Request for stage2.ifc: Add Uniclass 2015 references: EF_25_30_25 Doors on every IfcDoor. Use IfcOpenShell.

First a look at what the model holds.

```python
import ifcopenshell

model = ifcopenshell.open("stage2.ifc")
print(model.schema)
print("classifications:", [c.Name for c in model.by_type("IfcClassification")])
for ifc_class in ("IfcDoor", "IfcRoof", "IfcStair", "IfcWall", "IfcWindow"):
    print(ifc_class, len(model.by_type(ifc_class)))
```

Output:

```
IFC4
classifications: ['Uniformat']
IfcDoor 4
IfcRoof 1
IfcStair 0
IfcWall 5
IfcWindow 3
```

```python
import ifcopenshell
import ifcopenshell.api.classification

model = ifcopenshell.open("stage2.ifc")

system = ifcopenshell.api.classification.add_classification(model, classification="Uniclass 2015")

codes = {
    "IfcDoor": ("EF_25_30_25", "Doors"),
}
for ifc_class, (code, name) in codes.items():
    products = model.by_type(ifc_class)
    ifcopenshell.api.classification.add_reference(
        model, products=products, classification=system, identification=code, name=name
    )
    print(code, len(products))

model.write("stage2-out.ifc")
```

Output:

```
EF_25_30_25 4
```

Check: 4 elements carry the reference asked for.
